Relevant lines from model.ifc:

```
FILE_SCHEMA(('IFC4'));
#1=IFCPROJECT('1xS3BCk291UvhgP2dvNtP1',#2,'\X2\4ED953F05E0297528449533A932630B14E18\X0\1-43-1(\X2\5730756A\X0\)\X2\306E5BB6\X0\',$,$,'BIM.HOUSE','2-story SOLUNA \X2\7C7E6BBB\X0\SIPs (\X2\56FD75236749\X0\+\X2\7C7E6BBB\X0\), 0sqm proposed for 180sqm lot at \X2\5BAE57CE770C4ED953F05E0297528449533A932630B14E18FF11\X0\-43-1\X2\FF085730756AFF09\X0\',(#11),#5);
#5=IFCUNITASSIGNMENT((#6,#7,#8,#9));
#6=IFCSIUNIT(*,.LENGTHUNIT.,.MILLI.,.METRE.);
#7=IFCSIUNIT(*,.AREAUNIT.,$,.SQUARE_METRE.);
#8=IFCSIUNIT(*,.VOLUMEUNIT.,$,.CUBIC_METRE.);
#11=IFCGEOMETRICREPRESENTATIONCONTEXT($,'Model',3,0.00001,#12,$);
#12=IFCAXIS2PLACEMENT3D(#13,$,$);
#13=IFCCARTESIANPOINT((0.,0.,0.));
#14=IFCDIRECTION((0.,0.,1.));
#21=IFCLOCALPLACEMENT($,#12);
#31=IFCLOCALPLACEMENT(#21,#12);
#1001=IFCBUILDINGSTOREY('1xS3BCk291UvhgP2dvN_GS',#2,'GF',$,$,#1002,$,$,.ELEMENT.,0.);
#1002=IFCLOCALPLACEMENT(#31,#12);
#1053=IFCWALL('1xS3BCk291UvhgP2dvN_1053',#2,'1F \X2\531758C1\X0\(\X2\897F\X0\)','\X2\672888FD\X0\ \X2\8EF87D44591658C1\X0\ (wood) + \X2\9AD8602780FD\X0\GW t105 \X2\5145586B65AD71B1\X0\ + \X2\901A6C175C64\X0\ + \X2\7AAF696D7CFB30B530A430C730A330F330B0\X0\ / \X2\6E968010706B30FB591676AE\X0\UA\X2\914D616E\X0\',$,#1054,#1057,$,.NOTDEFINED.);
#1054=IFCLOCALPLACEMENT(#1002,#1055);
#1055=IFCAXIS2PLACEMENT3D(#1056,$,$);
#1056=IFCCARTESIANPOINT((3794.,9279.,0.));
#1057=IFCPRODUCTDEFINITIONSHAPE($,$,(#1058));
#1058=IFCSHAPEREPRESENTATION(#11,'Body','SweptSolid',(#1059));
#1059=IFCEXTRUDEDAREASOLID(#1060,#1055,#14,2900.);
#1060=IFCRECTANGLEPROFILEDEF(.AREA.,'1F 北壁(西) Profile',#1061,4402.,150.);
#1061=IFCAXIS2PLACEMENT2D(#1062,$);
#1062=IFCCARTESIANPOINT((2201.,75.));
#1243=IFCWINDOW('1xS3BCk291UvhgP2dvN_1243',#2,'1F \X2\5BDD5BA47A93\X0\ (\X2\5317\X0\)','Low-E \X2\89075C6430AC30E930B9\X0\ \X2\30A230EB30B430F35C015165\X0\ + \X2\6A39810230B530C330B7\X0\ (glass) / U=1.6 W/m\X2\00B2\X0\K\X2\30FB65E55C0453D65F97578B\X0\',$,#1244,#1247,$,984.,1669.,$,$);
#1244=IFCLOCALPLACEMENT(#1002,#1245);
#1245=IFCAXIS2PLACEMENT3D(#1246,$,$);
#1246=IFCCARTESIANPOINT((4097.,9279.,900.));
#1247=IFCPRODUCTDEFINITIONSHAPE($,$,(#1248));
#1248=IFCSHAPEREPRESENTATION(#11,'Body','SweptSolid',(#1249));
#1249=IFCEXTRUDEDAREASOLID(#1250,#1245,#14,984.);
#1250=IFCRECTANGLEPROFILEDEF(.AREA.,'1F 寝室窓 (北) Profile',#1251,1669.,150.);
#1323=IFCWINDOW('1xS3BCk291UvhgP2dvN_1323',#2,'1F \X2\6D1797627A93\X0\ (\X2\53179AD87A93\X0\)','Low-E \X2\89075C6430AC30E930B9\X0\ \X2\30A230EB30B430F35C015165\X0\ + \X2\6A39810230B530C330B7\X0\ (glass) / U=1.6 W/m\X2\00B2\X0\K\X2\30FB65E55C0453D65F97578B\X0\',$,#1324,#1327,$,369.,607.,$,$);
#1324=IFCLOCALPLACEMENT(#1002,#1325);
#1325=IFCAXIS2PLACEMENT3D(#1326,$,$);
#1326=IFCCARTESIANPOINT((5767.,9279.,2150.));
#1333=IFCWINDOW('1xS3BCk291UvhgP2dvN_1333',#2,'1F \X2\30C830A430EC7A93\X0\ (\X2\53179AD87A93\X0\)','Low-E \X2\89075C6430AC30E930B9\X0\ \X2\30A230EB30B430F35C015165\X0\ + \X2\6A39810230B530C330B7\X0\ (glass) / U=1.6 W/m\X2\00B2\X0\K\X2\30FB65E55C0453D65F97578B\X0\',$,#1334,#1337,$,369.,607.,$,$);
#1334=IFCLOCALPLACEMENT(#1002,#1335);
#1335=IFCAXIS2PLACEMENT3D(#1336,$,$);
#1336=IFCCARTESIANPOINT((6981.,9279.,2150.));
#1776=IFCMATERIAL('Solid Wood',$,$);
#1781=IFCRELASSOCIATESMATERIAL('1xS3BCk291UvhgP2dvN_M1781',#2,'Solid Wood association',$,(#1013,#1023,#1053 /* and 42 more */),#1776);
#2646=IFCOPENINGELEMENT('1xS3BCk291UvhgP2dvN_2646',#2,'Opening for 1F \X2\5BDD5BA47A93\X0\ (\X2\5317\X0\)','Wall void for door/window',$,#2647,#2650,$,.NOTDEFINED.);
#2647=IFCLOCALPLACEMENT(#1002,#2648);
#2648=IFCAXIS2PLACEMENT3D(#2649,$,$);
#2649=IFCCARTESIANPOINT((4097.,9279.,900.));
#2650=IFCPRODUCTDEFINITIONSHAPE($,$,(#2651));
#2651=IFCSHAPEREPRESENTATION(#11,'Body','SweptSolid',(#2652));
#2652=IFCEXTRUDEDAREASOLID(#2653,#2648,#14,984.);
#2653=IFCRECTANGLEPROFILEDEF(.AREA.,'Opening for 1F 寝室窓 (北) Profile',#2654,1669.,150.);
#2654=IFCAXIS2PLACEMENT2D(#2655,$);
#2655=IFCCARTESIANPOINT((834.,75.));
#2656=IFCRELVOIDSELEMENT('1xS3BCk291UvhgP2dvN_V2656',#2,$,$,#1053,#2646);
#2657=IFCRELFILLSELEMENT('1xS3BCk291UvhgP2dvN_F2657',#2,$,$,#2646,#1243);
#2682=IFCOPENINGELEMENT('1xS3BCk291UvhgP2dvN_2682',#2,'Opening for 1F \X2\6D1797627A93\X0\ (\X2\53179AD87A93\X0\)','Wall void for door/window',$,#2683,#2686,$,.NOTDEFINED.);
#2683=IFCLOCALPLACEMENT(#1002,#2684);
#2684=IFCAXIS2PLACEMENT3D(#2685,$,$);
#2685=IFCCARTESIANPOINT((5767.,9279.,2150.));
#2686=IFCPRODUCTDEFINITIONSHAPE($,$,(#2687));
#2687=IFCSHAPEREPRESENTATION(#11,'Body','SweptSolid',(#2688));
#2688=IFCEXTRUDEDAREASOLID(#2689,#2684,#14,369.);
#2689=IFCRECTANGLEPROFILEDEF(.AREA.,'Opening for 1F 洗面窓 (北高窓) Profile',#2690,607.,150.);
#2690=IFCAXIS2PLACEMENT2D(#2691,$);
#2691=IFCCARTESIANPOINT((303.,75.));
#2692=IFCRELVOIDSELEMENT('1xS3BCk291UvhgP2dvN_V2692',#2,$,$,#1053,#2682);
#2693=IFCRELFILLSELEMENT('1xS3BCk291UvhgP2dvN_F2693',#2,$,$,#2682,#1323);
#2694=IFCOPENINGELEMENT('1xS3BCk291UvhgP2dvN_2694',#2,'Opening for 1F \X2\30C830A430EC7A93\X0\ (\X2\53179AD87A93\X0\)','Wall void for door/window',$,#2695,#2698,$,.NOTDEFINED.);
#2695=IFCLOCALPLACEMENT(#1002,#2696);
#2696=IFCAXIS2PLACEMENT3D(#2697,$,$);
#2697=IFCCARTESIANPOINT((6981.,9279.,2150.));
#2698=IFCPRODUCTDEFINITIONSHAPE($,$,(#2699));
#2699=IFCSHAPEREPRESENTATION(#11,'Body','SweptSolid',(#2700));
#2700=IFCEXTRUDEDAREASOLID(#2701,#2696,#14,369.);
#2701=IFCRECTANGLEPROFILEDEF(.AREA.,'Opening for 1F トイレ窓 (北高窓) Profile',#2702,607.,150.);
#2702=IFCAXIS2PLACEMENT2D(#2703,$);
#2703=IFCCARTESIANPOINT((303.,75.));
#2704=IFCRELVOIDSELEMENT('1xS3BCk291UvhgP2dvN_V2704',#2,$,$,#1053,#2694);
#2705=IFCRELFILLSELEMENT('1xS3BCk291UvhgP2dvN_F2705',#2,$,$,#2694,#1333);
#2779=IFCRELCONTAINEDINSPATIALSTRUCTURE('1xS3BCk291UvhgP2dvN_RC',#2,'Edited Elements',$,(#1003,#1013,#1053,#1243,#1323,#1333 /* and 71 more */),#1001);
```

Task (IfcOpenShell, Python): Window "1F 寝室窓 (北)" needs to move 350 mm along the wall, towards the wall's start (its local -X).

```python
import ifcopenshell
import ifcopenshell.api.geometry
import ifcopenshell.util.placement

model = ifcopenshell.open("model.ifc")

window = model.by_guid("1xS3BCk291UvhgP2dvN_1243")
opening = window.FillsVoids[0].RelatingOpeningElement
wall = opening.VoidsElements[0].RelatingBuildingElement

wall_matrix = ifcopenshell.util.placement.get_local_placement(wall.ObjectPlacement)
shift = wall_matrix[:3, 0] * -350.0
before = ifcopenshell.util.placement.get_local_placement(window.ObjectPlacement)[:3, 3].copy()

# The window is not placed relative to its opening, so move both.
for product in (opening, window):
    matrix = ifcopenshell.util.placement.get_local_placement(product.ObjectPlacement)
    matrix[:3, 3] += shift
    ifcopenshell.api.geometry.edit_object_placement(model, product=product, matrix=matrix, is_si=False)

after = ifcopenshell.util.placement.get_local_placement(window.ObjectPlacement)[:3, 3]
print("window moved by", (after - before).round(3) + 0.0)

model.write("model-out.ifc")
```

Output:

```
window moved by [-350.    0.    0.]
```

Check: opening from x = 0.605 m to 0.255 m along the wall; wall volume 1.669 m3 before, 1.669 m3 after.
